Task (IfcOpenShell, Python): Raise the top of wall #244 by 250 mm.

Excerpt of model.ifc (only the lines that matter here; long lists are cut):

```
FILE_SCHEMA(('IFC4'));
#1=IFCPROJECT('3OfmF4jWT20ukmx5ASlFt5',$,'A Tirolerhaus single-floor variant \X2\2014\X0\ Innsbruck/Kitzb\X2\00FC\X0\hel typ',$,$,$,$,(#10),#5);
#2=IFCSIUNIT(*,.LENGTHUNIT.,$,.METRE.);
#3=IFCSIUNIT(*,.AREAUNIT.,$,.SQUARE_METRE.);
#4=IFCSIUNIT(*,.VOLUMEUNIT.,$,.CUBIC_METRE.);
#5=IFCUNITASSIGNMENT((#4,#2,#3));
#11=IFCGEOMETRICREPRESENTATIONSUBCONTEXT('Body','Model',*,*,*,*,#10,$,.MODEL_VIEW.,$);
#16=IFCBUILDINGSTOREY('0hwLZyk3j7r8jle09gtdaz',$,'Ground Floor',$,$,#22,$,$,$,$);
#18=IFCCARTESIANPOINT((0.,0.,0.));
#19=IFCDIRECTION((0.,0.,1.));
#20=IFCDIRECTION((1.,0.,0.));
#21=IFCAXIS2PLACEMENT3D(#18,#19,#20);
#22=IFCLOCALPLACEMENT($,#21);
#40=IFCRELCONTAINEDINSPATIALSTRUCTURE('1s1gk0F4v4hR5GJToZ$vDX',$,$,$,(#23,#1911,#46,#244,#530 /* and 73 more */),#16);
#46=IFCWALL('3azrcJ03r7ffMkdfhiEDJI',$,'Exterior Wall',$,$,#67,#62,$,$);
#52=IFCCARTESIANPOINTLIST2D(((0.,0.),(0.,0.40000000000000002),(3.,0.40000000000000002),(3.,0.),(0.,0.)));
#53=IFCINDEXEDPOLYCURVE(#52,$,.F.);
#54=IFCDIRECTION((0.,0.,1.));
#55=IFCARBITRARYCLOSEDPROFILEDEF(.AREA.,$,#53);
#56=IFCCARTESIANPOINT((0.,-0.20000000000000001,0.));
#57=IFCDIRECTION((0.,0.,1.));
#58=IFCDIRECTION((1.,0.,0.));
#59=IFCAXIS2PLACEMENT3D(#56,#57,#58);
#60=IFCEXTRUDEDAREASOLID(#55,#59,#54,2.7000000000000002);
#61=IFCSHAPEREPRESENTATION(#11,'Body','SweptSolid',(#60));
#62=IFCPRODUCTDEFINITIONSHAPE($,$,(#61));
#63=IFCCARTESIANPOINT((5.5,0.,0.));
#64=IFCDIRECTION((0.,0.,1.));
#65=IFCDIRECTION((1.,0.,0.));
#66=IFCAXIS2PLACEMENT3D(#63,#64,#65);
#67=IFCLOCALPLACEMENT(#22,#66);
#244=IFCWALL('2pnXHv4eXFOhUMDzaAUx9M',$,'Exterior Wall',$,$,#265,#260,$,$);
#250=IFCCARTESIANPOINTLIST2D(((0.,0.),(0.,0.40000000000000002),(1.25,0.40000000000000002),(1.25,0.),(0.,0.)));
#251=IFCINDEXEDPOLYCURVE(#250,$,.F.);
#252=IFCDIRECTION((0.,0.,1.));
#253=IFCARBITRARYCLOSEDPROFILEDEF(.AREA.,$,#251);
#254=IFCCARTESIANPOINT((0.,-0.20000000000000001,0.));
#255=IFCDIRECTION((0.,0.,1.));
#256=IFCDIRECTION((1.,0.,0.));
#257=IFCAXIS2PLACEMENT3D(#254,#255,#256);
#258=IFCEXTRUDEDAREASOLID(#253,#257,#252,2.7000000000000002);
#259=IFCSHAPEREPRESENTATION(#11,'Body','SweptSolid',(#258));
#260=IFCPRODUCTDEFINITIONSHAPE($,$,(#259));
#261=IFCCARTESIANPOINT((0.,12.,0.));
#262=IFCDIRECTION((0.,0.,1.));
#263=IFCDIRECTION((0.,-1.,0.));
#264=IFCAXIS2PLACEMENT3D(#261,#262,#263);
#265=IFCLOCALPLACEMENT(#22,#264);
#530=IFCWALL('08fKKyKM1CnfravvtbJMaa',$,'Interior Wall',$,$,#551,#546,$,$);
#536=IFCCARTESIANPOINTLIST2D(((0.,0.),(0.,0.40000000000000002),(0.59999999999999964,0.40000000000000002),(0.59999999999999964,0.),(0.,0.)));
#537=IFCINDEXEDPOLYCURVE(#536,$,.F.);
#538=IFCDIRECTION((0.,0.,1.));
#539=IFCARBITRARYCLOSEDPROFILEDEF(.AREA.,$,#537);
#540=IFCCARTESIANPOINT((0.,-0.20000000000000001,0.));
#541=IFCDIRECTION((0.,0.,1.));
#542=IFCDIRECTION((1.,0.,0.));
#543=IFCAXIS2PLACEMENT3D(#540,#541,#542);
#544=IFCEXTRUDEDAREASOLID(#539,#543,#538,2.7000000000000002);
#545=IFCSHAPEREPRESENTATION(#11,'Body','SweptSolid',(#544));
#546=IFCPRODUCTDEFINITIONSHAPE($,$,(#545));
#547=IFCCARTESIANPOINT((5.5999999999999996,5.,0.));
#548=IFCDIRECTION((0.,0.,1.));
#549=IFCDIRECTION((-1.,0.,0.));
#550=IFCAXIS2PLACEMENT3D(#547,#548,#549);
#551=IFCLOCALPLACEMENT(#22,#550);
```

```python
import ifcopenshell
import ifcopenshell.geom
import ifcopenshell.util.representation
import ifcopenshell.util.shape

model = ifcopenshell.open("model.ifc")
settings = ifcopenshell.geom.settings()


def volume(element):
    """Net volume in cubic metres, openings subtracted."""
    shape = ifcopenshell.geom.create_shape(settings, element)
    return ifcopenshell.util.shape.get_volume(shape.geometry)


wall = model.by_guid("2pnXHv4eXFOhUMDzaAUx9M")
before = volume(wall)

body = ifcopenshell.util.representation.get_representation(wall, "Model", "Body")
solid = body.Items[0]
old_height = solid.Depth
solid.Depth += 0.25
after = volume(wall)

print(f"height {old_height:g} -> {solid.Depth:g}, volume {before:.3f} -> {after:.3f} m3")

model.write("model_v2.ifc")
```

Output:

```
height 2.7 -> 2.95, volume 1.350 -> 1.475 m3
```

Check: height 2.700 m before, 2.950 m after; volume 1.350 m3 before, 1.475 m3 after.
